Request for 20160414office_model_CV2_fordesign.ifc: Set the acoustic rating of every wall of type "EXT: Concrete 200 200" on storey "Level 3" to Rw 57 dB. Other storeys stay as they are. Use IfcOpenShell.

First a look at what the model holds.

```python
import ifcopenshell
import ifcopenshell.util.element

model = ifcopenshell.open("20160414office_model_CV2_fordesign.ifc")
print(model.schema)
storey = next(s for s in model.by_type("IfcBuildingStorey") if s.Name == "Level 3")
walls = [e for e in ifcopenshell.util.element.get_decomposition(storey) if e.is_a("IfcWall")]
seen = {}
for e in walls:
    element_type = ifcopenshell.util.element.get_type(e)
    key = (element_type.Name if element_type != e and element_type else None, ifcopenshell.util.element.get_pset(e, "Pset_WallCommon", "AcousticRating"))
    seen[key] = seen.get(key, 0) + 1
for (name, value), count in sorted(seen.items(), key=str):
    print(count, "x", name, "|", value)
```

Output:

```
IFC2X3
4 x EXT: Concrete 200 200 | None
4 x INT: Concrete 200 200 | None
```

```python
import ifcopenshell
import ifcopenshell.api.pset
import ifcopenshell.util.element

model = ifcopenshell.open("20160414office_model_CV2_fordesign.ifc")

storey = next(s for s in model.by_type("IfcBuildingStorey") if s.Name == "Level 3")
walls = [e for e in ifcopenshell.util.element.get_decomposition(storey) if e.is_a("IfcWall")]

count = 0
for e in walls:
    element_type = ifcopenshell.util.element.get_type(e)
    if element_type in (None, e) or element_type.Name != "EXT: Concrete 200 200":
        continue
    # add_pset returns the element's existing set when there is one.
    pset = ifcopenshell.api.pset.add_pset(model, product=e, name="Pset_WallCommon")
    ifcopenshell.api.pset.edit_pset(model, pset=pset, properties={"AcousticRating": "Rw 57 dB"})
    count += 1

print(count, "walls updated")

model.write("20160414office_model_CV2_fordesign_edited.ifc")
```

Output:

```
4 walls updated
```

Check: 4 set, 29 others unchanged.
